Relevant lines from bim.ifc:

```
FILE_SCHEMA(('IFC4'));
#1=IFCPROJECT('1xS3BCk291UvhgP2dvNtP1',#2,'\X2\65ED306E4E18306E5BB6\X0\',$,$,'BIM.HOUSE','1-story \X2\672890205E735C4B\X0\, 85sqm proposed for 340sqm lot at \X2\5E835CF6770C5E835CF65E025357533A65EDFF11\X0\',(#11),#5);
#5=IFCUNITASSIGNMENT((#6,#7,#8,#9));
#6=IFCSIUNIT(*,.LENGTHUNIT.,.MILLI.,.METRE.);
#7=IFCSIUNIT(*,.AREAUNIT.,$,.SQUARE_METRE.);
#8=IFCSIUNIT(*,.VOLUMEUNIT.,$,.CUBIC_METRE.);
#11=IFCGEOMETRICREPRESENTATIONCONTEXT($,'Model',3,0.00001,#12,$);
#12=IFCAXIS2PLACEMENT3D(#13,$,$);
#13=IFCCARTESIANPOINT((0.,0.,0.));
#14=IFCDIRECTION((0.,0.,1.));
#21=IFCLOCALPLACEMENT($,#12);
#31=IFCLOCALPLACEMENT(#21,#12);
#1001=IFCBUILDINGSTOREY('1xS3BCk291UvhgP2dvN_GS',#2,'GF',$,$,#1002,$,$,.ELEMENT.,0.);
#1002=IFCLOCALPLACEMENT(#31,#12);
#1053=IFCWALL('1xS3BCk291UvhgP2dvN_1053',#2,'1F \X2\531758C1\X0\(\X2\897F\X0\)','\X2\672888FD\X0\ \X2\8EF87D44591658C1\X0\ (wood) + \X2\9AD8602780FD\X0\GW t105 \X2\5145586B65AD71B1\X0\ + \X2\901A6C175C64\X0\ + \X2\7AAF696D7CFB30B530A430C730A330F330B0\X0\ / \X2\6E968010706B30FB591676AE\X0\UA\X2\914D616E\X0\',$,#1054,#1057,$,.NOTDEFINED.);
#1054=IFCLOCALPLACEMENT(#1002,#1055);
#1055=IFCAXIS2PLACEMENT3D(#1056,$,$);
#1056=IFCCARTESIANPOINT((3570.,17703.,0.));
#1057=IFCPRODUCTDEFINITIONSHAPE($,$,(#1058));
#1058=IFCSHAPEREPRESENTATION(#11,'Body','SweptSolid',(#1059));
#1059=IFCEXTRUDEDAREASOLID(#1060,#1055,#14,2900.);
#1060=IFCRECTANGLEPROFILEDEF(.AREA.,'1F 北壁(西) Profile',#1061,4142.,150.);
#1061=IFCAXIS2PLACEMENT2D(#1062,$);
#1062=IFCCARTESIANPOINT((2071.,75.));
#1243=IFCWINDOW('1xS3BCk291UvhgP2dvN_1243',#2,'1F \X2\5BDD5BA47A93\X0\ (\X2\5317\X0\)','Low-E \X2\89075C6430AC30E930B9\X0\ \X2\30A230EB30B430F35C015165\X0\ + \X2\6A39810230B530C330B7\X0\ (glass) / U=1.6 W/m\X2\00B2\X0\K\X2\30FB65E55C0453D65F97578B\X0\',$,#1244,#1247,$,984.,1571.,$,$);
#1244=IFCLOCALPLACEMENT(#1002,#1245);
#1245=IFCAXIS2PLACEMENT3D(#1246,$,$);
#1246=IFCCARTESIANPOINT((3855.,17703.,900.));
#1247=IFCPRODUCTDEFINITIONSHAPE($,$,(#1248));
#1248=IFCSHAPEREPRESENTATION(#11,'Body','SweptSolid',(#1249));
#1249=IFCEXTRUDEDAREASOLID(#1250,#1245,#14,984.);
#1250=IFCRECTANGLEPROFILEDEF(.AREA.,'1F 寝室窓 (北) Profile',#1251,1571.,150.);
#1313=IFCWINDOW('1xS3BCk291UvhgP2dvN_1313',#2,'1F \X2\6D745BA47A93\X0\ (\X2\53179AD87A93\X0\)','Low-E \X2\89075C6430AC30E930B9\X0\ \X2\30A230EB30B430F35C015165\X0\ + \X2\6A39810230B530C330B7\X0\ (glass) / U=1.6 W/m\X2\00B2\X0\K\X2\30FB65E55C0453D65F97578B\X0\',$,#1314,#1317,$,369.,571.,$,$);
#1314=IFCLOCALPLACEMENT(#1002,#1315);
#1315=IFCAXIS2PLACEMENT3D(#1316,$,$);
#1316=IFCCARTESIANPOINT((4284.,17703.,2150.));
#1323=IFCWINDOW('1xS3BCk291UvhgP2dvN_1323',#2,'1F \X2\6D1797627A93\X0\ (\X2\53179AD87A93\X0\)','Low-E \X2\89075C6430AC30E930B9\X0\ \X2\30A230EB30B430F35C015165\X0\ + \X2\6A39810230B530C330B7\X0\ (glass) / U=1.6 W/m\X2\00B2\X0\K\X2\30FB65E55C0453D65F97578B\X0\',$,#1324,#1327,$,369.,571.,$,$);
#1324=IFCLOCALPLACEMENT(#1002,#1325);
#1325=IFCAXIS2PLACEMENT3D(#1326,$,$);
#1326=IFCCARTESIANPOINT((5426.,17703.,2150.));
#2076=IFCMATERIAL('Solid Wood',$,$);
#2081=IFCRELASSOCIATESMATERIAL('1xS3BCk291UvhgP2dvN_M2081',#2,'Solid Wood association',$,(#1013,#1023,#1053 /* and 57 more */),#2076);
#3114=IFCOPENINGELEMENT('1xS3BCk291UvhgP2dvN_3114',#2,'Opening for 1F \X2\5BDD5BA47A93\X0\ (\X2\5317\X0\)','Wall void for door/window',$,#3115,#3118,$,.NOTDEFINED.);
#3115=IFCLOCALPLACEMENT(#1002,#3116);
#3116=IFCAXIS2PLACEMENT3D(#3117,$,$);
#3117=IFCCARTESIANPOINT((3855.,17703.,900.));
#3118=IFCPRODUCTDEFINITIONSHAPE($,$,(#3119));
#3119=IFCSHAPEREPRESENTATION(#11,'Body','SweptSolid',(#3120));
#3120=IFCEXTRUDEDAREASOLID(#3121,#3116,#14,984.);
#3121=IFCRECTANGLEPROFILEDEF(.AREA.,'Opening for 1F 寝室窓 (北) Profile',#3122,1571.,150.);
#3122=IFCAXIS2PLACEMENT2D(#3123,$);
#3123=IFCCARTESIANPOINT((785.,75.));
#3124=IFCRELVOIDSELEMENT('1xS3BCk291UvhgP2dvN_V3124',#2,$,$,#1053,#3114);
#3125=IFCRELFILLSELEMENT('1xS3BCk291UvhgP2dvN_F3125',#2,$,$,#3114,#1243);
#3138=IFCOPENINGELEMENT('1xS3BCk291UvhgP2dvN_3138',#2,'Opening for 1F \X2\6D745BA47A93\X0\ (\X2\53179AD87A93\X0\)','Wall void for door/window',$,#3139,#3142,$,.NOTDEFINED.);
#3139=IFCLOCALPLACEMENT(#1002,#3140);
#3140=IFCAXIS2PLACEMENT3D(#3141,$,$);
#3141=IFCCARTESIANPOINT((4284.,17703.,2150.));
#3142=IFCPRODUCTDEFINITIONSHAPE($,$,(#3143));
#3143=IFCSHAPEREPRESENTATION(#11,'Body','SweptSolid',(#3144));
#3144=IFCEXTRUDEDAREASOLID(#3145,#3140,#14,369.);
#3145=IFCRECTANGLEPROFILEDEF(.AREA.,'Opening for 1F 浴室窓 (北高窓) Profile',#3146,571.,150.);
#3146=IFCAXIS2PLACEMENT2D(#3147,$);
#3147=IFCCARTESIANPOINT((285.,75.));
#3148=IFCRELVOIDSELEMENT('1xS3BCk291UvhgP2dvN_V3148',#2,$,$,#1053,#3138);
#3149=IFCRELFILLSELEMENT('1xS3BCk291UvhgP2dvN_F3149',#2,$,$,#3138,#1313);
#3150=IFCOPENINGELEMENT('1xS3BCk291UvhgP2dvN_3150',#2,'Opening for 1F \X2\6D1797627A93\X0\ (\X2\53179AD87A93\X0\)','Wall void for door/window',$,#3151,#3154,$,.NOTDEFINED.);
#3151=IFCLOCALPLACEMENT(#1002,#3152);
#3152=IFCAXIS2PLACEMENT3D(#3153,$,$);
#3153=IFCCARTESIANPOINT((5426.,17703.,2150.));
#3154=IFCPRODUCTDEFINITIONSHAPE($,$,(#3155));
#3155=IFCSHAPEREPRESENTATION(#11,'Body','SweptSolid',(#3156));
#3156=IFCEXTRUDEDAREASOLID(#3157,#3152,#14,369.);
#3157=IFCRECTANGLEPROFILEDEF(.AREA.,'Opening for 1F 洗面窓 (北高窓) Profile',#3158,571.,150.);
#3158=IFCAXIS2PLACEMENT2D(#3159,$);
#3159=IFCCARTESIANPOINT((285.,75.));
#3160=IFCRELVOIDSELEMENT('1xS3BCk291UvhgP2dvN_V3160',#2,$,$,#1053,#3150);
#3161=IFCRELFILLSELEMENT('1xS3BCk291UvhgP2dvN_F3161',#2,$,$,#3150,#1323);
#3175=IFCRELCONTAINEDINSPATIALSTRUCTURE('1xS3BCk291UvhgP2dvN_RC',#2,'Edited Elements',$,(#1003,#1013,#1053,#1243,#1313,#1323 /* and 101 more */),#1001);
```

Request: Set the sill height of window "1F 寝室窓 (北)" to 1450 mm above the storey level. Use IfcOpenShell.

```python
import numpy as np
import ifcopenshell
import ifcopenshell.api.geometry
import ifcopenshell.geom
import ifcopenshell.util.element
import ifcopenshell.util.placement
import ifcopenshell.util.shape
import ifcopenshell.util.unit

model = ifcopenshell.open("bim.ifc")
unit_scale = ifcopenshell.util.unit.calculate_unit_scale(model)

window = model.by_guid("1xS3BCk291UvhgP2dvN_1243")
opening = window.FillsVoids[0].RelatingOpeningElement
storey = ifcopenshell.util.element.get_container(window, ifc_class="IfcBuildingStorey")
level = ifcopenshell.util.placement.get_local_placement(storey.ObjectPlacement)[2, 3]

# The opening's origin need not be at the sill, so measure its lowest point.
shape = ifcopenshell.geom.create_shape(ifcopenshell.geom.settings(), opening)
bottom = ifcopenshell.util.shape.get_shape_bottom_elevation(shape, shape.geometry) / unit_scale
dz = level + 1.45 / unit_scale - bottom

shift = np.array([0.0, 0.0, dz])
# The window is not placed relative to its opening, so move both.
for product in (opening, window):
    matrix = ifcopenshell.util.placement.get_local_placement(product.ObjectPlacement)
    matrix[:3, 3] += shift
    ifcopenshell.api.geometry.edit_object_placement(model, product=product, matrix=matrix, is_si=False)

print(f"moved by {dz * unit_scale:+.3f} m")

model.write("bim_rev.ifc")
```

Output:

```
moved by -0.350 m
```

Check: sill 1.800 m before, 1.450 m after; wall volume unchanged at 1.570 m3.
